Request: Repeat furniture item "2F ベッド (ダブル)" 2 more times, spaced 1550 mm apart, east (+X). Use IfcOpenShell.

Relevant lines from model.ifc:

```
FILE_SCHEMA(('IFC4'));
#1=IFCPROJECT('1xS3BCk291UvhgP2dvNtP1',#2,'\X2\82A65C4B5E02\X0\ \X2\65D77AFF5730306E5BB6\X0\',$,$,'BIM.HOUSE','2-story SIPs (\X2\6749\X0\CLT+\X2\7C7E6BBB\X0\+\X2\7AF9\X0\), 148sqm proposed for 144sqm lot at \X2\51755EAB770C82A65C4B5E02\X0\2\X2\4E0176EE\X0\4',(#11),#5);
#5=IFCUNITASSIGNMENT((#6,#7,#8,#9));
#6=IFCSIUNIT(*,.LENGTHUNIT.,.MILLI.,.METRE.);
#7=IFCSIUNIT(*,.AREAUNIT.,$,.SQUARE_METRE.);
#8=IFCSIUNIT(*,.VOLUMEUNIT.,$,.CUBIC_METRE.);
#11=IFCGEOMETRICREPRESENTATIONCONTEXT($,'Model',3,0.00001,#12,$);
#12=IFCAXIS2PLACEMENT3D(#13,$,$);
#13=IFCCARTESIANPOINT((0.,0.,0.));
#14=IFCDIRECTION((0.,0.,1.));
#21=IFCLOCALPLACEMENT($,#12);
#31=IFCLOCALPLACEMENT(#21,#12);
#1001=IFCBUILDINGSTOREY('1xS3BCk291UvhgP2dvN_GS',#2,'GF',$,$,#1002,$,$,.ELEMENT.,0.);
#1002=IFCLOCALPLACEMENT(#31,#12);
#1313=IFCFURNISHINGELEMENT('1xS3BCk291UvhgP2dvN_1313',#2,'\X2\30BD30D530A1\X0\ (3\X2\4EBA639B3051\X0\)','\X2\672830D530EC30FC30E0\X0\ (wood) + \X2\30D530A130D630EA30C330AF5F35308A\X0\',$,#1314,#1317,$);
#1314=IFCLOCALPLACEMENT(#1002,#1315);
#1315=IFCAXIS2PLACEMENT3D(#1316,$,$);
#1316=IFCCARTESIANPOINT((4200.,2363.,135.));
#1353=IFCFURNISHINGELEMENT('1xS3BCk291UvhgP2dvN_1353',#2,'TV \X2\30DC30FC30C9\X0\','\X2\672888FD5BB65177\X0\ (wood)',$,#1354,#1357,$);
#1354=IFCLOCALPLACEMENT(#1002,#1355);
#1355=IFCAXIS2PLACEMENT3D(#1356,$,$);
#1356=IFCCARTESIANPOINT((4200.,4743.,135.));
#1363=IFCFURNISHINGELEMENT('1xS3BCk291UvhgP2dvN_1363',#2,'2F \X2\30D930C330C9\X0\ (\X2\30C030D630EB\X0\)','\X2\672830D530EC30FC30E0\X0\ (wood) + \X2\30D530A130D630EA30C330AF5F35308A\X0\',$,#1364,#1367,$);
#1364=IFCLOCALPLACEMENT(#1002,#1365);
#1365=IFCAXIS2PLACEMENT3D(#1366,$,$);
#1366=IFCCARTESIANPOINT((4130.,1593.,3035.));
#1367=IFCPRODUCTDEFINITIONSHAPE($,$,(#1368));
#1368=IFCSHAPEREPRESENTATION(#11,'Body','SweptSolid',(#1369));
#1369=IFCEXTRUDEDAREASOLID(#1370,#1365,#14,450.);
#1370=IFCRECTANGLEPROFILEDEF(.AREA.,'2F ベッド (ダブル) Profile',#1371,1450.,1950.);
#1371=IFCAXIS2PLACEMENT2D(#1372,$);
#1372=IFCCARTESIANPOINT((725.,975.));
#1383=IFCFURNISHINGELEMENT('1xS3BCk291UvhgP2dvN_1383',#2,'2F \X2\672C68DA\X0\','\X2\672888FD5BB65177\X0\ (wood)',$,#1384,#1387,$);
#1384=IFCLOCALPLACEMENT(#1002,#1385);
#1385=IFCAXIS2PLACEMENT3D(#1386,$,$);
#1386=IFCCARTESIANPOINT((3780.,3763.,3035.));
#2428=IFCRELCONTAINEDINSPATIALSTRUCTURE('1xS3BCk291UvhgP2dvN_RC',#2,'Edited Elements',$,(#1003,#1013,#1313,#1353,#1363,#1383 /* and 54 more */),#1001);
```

```python
import numpy as np
import ifcopenshell
import ifcopenshell.api.geometry
import ifcopenshell.api.root
import ifcopenshell.util.element
import ifcopenshell.util.placement

model = ifcopenshell.open("model.ifc")


def reuse_history(source, copy):
    """copy_class also copies each property set's owner history, people and application; keep the originals."""
    for rel in copy.IsDefinedBy:
        if rel.is_a("IfcRelDefinesByProperties") and (history := rel.RelatingPropertyDefinition.OwnerHistory):
            rel.RelatingPropertyDefinition.OwnerHistory = source.OwnerHistory
            ifcopenshell.util.element.remove_deep2(model, history)


source = model.by_id(1363)
base = ifcopenshell.util.placement.get_local_placement(source.ObjectPlacement)
step = np.array([1.0, 0.0, 0.0]) * 1550.0

for i in range(1, 3):
    copy = ifcopenshell.api.root.copy_class(model, product=source)
    copy.Representation = ifcopenshell.util.element.copy_deep(
        model, source.Representation, exclude=["IfcGeometricRepresentationContext", "IfcRepresentationMap"]
    )
    reuse_history(source, copy)
    matrix = base.copy()
    matrix[:3, 3] += i * step
    print("added at", matrix[:3, 3].round(3) + 0.0)
    ifcopenshell.api.geometry.edit_object_placement(model, product=copy, matrix=matrix, is_si=False)

model.write("model_edited.ifc")
```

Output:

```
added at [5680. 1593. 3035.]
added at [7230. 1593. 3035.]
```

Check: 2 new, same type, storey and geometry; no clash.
